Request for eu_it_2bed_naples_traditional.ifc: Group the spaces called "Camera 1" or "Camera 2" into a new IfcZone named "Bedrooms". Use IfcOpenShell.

First a look at what the model holds.

```python
import ifcopenshell

model = ifcopenshell.open("eu_it_2bed_naples_traditional.ifc")
print(model.schema)
seen = {}
for space in model.by_type("IfcSpace"):
    seen[space.LongName] = seen.get(space.LongName, 0) + 1
for name, count in sorted(seen.items(), key=str):
    print(count, "x", name)
print("zones:", [z.Name for z in model.by_type("IfcZone")][:20])
```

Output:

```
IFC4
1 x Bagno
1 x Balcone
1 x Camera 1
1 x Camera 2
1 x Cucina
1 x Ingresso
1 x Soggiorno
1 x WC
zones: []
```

```python
import ifcopenshell
import ifcopenshell.api.group
import ifcopenshell.api.root

model = ifcopenshell.open("eu_it_2bed_naples_traditional.ifc")

names = {"Camera 1", "Camera 2"}
spaces = [s for s in model.by_type("IfcSpace") if s.LongName in names]

zone = ifcopenshell.api.root.create_entity(model, ifc_class="IfcZone", name="Bedrooms")
ifcopenshell.api.group.assign_group(model, products=spaces, group=zone)
print(len(spaces), "spaces in", zone.Name)

model.write("eu_it_2bed_naples_traditional_updated.ifc")
```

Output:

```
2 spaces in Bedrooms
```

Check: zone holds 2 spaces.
